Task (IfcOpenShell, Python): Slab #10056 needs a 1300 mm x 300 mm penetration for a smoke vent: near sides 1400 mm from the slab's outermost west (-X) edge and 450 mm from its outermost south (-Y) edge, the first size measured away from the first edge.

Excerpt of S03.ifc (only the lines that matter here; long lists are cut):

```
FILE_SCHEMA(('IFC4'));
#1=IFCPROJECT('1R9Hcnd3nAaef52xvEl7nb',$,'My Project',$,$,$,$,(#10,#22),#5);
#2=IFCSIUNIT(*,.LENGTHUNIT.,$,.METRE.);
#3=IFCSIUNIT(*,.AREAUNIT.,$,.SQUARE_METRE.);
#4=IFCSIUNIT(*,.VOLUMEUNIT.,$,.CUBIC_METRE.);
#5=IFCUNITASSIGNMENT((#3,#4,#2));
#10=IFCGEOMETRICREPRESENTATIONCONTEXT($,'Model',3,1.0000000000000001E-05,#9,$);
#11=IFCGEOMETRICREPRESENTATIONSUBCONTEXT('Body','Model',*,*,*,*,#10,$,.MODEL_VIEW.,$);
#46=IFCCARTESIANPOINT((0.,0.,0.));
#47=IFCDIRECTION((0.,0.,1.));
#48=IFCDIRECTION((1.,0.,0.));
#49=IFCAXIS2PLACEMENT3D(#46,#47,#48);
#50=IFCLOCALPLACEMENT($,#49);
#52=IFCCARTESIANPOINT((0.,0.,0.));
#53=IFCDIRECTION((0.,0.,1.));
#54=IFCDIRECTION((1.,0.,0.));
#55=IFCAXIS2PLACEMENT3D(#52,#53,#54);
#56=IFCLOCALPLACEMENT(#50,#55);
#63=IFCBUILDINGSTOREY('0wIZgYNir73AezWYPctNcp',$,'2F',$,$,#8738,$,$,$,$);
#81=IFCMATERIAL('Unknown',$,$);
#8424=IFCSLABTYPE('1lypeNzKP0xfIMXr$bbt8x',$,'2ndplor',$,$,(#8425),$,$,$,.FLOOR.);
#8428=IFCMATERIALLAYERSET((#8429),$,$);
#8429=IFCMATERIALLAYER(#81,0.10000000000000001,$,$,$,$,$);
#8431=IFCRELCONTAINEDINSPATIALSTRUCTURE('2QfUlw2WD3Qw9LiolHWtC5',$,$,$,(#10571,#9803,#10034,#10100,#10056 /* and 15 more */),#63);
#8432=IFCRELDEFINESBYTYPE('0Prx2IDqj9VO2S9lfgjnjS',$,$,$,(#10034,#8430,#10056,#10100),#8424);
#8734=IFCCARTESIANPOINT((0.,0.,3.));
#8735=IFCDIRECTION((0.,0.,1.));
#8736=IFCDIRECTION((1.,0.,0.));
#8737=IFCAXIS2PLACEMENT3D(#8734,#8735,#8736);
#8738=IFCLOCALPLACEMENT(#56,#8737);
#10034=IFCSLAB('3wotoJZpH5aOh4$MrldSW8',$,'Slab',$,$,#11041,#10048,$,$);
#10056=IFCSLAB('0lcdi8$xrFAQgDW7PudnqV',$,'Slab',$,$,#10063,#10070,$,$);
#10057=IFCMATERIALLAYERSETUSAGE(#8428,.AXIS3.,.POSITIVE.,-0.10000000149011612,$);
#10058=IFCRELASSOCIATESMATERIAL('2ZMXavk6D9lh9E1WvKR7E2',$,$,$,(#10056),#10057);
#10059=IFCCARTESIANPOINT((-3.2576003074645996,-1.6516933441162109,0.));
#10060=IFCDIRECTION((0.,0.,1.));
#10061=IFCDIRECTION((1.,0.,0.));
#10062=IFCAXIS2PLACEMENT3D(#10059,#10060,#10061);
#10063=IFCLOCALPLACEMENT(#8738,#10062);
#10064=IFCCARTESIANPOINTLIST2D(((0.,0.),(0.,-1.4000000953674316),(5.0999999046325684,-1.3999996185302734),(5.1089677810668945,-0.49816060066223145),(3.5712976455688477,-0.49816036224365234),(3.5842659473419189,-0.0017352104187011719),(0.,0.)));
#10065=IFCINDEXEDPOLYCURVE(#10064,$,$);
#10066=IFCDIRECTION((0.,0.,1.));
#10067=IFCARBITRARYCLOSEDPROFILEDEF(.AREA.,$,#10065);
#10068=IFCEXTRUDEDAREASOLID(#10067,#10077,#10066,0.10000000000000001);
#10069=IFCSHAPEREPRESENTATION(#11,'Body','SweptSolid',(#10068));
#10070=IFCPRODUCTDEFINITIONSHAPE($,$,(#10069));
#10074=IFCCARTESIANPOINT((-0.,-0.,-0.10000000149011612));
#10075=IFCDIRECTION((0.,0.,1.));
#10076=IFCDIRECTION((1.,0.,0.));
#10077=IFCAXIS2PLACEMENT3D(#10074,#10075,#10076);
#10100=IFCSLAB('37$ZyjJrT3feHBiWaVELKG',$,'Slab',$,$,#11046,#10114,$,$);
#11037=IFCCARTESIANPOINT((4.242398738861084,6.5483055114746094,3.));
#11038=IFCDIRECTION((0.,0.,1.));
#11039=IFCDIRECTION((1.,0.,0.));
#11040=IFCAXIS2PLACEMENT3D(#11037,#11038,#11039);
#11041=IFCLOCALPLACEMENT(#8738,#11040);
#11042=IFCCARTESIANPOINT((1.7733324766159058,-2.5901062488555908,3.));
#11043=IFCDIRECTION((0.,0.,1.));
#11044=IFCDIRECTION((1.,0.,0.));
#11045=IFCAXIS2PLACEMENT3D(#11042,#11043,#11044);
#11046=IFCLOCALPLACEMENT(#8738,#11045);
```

```python
import numpy as np
import ifcopenshell
import ifcopenshell.api.feature
import ifcopenshell.api.geometry
import ifcopenshell.api.root
import ifcopenshell.geom
import ifcopenshell.util.placement
import ifcopenshell.util.representation
import ifcopenshell.util.shape
import ifcopenshell.util.unit

model = ifcopenshell.open("S03.ifc")
unit_scale = ifcopenshell.util.unit.calculate_unit_scale(model)
settings = ifcopenshell.geom.settings()


def volume(element):
    """Net volume in cubic metres, openings subtracted."""
    shape = ifcopenshell.geom.create_shape(settings, element)
    return ifcopenshell.util.shape.get_volume(shape.geometry)


slab = model.by_guid("0lcdi8$xrFAQgDW7PudnqV")
before = volume(slab)

# Extent in the slab's own axes, in metres. The edges named are its -X and -Y sides.
slab_shape = ifcopenshell.geom.create_shape(settings, slab)
vertices = ifcopenshell.util.shape.get_vertices(slab_shape.geometry)
x_min, y_min, bottom = vertices.min(axis=0)
top = vertices[:, 2].max()

opening = ifcopenshell.api.root.create_entity(model, ifc_class="IfcOpeningElement", name="Smoke vent opening", predefined_type="OPENING")
context = ifcopenshell.util.representation.get_context(model, "Model", "Body", "MODEL_VIEW")
width, depth = 1.3, 0.3
outline = [(0.0, 0.0), (width, 0.0), (width, depth), (0.0, depth), (0.0, 0.0)]
# Overshoot both faces by 50 mm so the cut is clean.
shape = ifcopenshell.api.geometry.add_slab_representation(
    model, context=context, depth=top - bottom + 0.1, polyline=outline
)
ifcopenshell.api.geometry.assign_representation(model, product=opening, representation=shape)

matrix = ifcopenshell.util.placement.get_local_placement(slab.ObjectPlacement)
matrix[:, 3] = matrix @ np.append(np.array([x_min + 1.4, y_min + 0.45, bottom - 0.05]) / unit_scale, 1.0)
ifcopenshell.api.geometry.edit_object_placement(model, product=opening, matrix=matrix, is_si=False)
ifcopenshell.api.feature.add_feature(model, feature=opening, element=slab)

after = volume(slab)

print(f"slab volume {before:.3f} -> {after:.3f} m3")

model.write("S03-out.ifc")
```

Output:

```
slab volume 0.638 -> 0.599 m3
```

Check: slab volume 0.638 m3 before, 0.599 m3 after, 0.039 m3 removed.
